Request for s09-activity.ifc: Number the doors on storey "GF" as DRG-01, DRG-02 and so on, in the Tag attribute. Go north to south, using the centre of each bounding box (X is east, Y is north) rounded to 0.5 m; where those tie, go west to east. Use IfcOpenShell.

First a look at what the model holds.

```python
import ifcopenshell
import ifcopenshell.util.element
import ifcopenshell.util.placement

model = ifcopenshell.open("s09-activity.ifc")
print(model.schema)
storey = next(s for s in model.by_type("IfcBuildingStorey") if s.Name == "GF")
doors = [e for e in ifcopenshell.util.element.get_decomposition(storey) if e.is_a("IfcDoor")]
for e in sorted(doors, key=lambda e: e.id()):
    origin = ifcopenshell.util.placement.get_local_placement(e.ObjectPlacement)[:3, 3]
    print(e.id(), e.Tag, e.Name, origin.round(2) + 0.0, sep=" | ")
```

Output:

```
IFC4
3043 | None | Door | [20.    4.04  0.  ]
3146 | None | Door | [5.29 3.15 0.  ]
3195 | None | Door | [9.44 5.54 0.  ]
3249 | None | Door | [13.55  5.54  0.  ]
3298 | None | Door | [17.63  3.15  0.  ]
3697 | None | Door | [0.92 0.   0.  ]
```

```python
import ifcopenshell
import ifcopenshell.geom
import ifcopenshell.util.element
import ifcopenshell.util.shape

model = ifcopenshell.open("s09-activity.ifc")
settings = ifcopenshell.geom.settings()
settings.set("use-world-coords", True)


def centre(element):
    shape = ifcopenshell.geom.create_shape(settings, element)
    return ifcopenshell.util.shape.get_bbox_centroid(shape.geometry)


storey = next(s for s in model.by_type("IfcBuildingStorey") if s.Name == "GF")
doors = [e for e in ifcopenshell.util.element.get_decomposition(storey) if e.is_a("IfcDoor")]

# Insertion points can sit at a corner or the storey origin, so sort by the geometry (in metres).
centres = {e: centre(e) for e in doors}
doors.sort(key=lambda e: (-round(centres[e][1] / 0.5), centres[e][0]))

for i, e in enumerate(doors, start=1):
    number = f"DRG-{i:02d}"
    e.Tag = number
    print(e.id(), number)

model.write("s09-activity-out.ifc")
```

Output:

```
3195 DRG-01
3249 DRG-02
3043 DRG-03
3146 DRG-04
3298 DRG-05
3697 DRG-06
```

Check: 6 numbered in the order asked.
